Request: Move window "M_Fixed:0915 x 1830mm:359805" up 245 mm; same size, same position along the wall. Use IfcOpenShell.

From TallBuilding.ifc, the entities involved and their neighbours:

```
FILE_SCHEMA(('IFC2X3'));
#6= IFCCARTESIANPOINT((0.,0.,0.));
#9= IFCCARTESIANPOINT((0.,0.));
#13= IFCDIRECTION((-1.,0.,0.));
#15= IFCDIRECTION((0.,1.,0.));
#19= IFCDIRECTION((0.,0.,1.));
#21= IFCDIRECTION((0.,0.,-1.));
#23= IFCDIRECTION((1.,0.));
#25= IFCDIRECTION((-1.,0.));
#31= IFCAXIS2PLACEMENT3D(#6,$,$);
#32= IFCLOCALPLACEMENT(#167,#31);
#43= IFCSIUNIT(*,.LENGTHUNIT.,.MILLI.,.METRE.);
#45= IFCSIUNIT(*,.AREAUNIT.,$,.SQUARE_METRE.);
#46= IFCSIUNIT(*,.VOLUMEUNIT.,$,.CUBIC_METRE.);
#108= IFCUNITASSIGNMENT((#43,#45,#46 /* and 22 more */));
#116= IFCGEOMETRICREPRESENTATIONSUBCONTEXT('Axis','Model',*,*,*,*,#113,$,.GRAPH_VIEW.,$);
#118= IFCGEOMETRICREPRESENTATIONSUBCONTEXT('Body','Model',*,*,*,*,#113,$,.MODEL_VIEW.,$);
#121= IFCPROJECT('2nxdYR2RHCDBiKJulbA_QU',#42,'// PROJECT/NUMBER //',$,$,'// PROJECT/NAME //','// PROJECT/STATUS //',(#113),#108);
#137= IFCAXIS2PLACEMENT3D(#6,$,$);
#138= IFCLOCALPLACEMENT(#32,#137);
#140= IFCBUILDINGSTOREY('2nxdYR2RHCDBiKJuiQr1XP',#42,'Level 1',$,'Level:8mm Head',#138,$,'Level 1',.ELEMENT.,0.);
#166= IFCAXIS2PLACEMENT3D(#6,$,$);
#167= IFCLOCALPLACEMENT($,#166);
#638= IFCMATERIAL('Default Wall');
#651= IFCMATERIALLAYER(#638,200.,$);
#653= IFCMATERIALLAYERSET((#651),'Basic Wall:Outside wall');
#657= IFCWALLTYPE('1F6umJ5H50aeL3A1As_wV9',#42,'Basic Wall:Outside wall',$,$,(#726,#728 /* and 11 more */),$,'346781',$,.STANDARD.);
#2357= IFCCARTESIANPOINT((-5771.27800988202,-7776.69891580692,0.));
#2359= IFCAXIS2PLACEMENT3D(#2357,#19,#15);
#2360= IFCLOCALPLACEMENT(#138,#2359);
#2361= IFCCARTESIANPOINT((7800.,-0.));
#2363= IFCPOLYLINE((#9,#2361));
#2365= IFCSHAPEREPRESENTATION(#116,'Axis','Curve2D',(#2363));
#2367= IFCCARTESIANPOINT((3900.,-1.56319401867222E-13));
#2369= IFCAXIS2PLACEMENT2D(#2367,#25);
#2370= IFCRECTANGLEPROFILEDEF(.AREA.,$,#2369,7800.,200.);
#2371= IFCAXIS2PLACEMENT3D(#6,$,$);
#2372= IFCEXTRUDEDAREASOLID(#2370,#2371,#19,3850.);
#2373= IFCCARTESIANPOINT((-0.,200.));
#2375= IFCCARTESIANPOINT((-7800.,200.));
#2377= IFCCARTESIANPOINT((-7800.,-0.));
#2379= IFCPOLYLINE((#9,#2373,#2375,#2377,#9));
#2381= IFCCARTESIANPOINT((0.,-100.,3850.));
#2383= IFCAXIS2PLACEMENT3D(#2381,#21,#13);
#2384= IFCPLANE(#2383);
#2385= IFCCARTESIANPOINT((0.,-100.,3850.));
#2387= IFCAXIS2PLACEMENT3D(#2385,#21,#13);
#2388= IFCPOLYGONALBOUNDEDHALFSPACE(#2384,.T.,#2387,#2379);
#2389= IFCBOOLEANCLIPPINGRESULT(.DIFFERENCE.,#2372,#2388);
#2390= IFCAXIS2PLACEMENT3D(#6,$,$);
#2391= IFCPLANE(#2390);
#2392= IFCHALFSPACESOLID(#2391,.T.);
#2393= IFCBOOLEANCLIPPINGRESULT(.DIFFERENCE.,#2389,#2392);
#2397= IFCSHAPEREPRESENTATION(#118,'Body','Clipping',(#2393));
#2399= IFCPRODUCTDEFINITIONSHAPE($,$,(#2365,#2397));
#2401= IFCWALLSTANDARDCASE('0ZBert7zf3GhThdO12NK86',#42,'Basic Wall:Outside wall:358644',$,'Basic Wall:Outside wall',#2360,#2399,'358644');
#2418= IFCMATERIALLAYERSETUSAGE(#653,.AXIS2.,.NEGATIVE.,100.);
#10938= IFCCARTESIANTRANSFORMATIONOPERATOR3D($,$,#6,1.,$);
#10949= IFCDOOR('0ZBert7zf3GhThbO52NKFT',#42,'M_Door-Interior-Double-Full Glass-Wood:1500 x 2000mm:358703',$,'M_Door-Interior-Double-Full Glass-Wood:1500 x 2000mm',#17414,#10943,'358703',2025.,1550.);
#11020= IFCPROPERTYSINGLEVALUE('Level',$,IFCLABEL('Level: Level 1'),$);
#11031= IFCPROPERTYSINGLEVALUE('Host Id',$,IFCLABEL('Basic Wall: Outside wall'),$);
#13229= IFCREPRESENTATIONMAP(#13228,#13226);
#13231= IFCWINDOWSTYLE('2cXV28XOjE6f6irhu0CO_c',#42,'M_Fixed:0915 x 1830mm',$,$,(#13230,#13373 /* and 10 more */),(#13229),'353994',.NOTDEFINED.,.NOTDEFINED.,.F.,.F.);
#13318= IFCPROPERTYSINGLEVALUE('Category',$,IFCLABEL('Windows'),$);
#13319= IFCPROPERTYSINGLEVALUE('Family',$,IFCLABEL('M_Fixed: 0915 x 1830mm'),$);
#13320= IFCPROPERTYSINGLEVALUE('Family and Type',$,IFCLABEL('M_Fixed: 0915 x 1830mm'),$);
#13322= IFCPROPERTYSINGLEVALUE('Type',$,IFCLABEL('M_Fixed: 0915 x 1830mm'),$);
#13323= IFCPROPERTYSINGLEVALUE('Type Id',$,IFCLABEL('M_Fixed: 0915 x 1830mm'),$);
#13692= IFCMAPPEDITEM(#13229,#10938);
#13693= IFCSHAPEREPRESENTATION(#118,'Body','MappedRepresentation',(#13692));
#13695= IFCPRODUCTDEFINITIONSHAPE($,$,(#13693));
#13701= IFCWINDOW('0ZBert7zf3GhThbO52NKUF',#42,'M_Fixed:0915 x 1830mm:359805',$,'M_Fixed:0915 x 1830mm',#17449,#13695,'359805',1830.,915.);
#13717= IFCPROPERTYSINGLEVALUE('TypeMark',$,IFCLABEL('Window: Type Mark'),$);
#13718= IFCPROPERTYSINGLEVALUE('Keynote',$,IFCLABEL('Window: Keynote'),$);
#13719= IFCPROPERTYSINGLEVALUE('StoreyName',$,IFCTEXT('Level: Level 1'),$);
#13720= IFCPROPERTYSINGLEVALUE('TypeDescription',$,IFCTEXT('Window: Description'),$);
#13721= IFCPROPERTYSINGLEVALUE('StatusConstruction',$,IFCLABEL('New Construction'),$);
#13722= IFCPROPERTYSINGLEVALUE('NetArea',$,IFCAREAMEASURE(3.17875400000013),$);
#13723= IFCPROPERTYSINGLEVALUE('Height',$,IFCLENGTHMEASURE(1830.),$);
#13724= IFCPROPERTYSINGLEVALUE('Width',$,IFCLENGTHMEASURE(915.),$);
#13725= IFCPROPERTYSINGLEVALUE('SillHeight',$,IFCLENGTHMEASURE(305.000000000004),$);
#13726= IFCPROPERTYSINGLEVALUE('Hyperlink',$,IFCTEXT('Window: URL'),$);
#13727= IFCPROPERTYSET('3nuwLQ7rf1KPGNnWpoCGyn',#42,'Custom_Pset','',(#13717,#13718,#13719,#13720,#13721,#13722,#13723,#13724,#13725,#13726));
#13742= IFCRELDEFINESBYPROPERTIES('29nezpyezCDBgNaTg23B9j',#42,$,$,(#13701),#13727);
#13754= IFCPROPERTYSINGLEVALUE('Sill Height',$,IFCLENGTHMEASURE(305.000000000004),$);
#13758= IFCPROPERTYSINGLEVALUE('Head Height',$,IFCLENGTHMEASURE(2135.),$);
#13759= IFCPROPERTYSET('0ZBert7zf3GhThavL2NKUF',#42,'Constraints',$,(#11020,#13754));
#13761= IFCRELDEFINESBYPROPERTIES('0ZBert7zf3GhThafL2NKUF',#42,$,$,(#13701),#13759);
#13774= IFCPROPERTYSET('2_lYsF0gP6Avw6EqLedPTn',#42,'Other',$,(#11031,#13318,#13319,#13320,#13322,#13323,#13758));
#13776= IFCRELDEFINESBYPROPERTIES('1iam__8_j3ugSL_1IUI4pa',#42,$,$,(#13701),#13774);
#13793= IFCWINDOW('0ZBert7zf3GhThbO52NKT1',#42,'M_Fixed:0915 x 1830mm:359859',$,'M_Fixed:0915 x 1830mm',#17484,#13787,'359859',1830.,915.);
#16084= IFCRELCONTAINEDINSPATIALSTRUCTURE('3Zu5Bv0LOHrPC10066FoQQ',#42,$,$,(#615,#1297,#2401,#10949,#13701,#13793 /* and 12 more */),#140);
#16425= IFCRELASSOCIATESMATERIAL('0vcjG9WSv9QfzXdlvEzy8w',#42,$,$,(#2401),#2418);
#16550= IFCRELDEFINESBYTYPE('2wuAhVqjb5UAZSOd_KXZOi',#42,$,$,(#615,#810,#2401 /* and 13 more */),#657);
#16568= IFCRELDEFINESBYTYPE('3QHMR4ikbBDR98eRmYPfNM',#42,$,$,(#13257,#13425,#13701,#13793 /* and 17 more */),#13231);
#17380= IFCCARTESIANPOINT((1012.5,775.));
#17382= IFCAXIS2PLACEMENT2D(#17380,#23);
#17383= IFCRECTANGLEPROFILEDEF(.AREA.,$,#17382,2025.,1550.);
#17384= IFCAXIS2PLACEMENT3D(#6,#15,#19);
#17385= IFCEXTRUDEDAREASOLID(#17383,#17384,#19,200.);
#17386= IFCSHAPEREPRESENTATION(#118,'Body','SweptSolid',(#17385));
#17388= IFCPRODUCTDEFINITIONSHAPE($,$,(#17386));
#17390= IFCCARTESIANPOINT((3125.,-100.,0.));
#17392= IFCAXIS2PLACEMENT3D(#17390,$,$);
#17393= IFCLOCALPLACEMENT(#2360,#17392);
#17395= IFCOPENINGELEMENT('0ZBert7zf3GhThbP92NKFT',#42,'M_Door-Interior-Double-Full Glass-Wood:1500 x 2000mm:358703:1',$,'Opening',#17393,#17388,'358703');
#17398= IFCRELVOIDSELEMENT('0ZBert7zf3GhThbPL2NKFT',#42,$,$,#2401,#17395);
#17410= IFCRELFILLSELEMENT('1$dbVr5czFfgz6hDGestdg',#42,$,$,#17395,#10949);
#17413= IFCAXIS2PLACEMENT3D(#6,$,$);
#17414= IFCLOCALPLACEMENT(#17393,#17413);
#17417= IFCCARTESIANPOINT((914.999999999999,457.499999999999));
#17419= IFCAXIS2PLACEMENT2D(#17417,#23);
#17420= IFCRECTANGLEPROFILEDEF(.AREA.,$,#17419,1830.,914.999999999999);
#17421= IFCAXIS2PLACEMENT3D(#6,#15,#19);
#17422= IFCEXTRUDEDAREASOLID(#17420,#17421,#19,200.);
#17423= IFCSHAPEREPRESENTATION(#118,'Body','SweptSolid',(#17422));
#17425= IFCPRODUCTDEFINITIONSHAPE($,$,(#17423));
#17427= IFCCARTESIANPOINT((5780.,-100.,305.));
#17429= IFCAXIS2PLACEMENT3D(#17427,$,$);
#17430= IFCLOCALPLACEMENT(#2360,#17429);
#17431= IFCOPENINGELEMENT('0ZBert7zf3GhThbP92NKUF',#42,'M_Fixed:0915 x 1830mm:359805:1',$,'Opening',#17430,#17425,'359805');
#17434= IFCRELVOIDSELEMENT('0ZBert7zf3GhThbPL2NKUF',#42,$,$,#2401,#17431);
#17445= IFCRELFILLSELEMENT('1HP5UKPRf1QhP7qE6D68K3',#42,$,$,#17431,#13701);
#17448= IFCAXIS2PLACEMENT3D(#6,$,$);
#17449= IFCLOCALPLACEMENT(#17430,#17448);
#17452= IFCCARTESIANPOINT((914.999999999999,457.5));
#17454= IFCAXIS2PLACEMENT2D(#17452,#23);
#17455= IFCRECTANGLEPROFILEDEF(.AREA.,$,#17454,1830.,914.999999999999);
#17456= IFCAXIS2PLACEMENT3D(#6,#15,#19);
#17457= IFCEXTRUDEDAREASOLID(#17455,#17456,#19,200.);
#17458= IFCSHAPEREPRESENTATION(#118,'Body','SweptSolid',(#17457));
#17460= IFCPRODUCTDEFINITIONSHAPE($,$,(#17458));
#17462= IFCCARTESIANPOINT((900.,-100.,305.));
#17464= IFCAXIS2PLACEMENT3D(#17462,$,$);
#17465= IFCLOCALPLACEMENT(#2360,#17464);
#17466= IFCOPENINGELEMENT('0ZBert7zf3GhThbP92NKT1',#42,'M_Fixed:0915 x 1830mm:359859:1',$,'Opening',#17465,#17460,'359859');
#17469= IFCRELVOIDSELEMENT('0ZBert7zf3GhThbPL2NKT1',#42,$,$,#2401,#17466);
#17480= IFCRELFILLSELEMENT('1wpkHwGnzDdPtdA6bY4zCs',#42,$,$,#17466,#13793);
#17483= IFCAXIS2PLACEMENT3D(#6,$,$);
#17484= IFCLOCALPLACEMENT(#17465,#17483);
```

```python
import numpy as np
import ifcopenshell
import ifcopenshell.api.geometry
import ifcopenshell.api.pset
import ifcopenshell.util.element
import ifcopenshell.util.placement
import ifcopenshell.util.unit

model = ifcopenshell.open("TallBuilding.ifc")
unit_scale = ifcopenshell.util.unit.calculate_unit_scale(model)

window = model.by_guid("0ZBert7zf3GhThbO52NKUF")
opening = window.FillsVoids[0].RelatingOpeningElement
dz = 245.0

shift = np.array([0.0, 0.0, dz])
# The window is placed relative to its opening, so it follows when the opening moves.
matrix = ifcopenshell.util.placement.get_local_placement(opening.ObjectPlacement)
matrix[:3, 3] += shift
ifcopenshell.api.geometry.edit_object_placement(
    model, product=opening, matrix=matrix, is_si=False, should_transform_children=True
)

# Keep the stored heights in step.
pset = model.by_id(ifcopenshell.util.element.get_pset(window, "Custom_Pset", should_inherit=False)["id"])
ifcopenshell.api.pset.edit_pset(model, pset=pset, properties={
    "SillHeight": model.create_entity("IfcLengthMeasure", ifcopenshell.util.element.get_pset(window, "Constraints", "Sill Height") + dz),
})
pset = model.by_id(ifcopenshell.util.element.get_pset(window, "Constraints", should_inherit=False)["id"])
ifcopenshell.api.pset.edit_pset(model, pset=pset, properties={
    "Sill Height": model.create_entity("IfcLengthMeasure", ifcopenshell.util.element.get_pset(window, "Constraints", "Sill Height") + dz),
})
pset = model.by_id(ifcopenshell.util.element.get_pset(window, "Other", should_inherit=False)["id"])
ifcopenshell.api.pset.edit_pset(model, pset=pset, properties={
    "Head Height": model.create_entity("IfcLengthMeasure", ifcopenshell.util.element.get_pset(window, "Other", "Head Height") + dz),
})

print(f"moved by {dz * unit_scale:+.3f} m")

model.write("TallBuilding-out.ifc")
```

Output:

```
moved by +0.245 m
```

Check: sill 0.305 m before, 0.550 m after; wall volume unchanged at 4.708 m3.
